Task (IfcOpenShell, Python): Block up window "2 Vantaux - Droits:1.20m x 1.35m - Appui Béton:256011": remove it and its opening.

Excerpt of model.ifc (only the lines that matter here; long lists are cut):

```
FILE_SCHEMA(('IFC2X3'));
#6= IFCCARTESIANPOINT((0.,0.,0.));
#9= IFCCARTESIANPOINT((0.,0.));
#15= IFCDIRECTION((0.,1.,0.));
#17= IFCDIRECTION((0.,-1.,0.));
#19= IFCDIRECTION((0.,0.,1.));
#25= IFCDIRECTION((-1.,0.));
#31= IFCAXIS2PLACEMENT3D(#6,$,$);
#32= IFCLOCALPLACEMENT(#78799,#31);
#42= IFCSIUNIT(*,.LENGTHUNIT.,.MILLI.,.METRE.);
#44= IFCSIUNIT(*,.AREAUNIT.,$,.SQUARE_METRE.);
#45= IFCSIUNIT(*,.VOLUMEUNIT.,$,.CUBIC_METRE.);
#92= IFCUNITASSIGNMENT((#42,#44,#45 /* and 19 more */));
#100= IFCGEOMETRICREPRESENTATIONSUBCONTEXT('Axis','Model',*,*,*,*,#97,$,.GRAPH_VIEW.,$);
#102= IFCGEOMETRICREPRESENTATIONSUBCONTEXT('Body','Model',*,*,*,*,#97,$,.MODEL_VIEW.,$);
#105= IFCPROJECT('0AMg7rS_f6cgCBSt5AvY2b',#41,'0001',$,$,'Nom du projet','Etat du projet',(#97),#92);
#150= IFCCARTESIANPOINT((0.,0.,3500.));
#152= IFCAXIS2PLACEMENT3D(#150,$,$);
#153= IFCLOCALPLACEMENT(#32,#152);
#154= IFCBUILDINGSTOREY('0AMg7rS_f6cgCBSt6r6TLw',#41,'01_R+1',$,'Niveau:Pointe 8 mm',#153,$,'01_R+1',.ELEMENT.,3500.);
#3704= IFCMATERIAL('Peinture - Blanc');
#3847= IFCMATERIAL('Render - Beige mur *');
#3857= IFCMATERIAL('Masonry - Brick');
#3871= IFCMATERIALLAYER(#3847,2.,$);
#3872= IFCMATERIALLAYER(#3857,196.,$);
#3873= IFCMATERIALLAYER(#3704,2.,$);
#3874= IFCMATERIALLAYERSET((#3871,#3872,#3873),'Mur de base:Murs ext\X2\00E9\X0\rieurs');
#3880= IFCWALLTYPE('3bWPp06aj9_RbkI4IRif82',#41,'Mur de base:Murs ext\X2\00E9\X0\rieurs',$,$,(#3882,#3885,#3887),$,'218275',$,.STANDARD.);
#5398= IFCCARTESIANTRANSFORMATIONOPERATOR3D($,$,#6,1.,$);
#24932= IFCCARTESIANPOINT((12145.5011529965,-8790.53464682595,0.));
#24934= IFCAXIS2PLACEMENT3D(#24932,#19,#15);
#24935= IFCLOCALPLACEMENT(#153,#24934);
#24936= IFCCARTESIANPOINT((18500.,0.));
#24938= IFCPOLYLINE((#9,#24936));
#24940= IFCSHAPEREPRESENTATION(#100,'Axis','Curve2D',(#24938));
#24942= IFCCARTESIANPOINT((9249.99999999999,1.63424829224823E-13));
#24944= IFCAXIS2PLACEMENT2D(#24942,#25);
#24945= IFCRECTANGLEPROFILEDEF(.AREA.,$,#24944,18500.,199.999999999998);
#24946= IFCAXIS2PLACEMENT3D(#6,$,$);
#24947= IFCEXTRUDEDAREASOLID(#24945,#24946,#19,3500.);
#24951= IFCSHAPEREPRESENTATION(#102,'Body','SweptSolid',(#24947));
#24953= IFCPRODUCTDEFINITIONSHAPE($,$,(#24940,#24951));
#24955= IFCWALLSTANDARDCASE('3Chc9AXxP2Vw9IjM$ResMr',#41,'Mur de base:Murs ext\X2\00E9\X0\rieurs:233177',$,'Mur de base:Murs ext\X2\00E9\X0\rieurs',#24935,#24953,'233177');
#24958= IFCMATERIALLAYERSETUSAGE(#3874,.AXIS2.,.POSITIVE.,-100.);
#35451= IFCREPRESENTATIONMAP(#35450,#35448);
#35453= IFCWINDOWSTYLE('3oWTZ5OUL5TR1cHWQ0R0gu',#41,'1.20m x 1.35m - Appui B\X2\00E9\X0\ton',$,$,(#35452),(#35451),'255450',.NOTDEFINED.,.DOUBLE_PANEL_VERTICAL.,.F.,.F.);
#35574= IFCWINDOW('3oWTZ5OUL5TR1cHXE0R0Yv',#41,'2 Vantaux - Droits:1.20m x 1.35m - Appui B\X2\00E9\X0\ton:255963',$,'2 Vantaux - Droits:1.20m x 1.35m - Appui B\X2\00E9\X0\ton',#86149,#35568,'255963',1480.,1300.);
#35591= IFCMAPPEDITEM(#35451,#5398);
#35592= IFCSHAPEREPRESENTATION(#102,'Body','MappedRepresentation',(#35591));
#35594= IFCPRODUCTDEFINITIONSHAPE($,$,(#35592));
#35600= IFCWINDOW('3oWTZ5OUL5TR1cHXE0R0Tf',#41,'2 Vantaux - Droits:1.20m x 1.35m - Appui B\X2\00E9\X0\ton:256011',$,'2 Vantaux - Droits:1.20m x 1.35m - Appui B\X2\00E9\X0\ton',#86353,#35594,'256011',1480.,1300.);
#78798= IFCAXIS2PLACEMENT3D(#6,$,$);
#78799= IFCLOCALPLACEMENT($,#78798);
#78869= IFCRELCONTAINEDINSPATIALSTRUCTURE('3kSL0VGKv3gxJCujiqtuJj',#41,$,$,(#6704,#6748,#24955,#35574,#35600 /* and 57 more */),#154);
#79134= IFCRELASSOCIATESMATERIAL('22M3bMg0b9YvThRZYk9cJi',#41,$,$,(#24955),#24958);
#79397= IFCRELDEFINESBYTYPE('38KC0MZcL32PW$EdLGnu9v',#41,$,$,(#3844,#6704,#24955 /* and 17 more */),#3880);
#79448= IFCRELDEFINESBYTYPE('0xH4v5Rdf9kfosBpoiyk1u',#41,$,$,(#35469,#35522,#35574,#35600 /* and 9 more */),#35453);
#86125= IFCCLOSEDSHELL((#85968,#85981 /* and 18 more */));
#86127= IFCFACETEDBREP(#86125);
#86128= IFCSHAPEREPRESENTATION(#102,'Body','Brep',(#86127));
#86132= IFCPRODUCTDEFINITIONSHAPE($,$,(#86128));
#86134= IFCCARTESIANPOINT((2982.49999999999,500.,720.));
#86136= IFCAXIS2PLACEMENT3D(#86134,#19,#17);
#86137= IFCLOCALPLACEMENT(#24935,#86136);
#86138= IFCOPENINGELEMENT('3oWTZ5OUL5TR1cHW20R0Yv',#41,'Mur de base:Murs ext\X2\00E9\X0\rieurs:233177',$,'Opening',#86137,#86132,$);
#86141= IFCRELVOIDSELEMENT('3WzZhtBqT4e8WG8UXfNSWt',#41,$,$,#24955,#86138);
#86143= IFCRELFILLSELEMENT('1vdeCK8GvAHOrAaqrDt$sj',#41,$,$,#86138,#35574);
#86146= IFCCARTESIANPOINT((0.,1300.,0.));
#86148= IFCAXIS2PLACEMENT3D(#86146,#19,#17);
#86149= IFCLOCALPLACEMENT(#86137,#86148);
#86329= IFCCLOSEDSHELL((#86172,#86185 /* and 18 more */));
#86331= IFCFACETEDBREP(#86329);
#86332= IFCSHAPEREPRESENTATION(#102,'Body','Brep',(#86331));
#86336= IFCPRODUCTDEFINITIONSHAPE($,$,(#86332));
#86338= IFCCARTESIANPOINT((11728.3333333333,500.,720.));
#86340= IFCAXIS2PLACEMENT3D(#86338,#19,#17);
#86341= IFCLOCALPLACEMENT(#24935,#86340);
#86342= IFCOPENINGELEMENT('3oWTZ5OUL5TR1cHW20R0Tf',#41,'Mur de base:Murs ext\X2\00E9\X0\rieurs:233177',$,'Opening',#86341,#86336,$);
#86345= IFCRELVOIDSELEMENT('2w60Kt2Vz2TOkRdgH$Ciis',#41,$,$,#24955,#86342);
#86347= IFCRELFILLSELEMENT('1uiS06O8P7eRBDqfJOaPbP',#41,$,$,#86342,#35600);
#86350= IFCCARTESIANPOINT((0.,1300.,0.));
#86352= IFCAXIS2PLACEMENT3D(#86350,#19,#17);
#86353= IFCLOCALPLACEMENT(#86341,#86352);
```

```python
import ifcopenshell
import ifcopenshell.api.feature
import ifcopenshell.api.root
import ifcopenshell.geom
import ifcopenshell.util.shape

model = ifcopenshell.open("model.ifc")
settings = ifcopenshell.geom.settings()


def volume(element):
    """Net volume in cubic metres, openings subtracted."""
    shape = ifcopenshell.geom.create_shape(settings, element)
    return ifcopenshell.util.shape.get_volume(shape.geometry)


window = model.by_guid("3oWTZ5OUL5TR1cHXE0R0Tf")
opening = window.FillsVoids[0].RelatingOpeningElement
wall = opening.VoidsElements[0].RelatingBuildingElement
before = volume(wall)

ifcopenshell.api.root.remove_product(model, product=window)
ifcopenshell.api.feature.remove_feature(model, feature=opening)

after = volume(wall)

print(f"wall volume {before:.3f} -> {after:.3f} m3")

model.write("model_edited.ifc")
```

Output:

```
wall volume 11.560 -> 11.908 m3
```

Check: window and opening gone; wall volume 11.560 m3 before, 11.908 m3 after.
